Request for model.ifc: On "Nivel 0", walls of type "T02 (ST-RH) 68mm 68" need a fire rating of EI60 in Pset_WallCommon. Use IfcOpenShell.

First a look at what the model holds.

```python
import ifcopenshell
import ifcopenshell.util.element

model = ifcopenshell.open("model.ifc")
print(model.schema)
storey = next(s for s in model.by_type("IfcBuildingStorey") if s.Name == "Nivel 0")
walls = [e for e in ifcopenshell.util.element.get_decomposition(storey) if e.is_a("IfcWall")]
seen = {}
for e in walls:
    element_type = ifcopenshell.util.element.get_type(e)
    key = (element_type.Name if element_type != e and element_type else None, ifcopenshell.util.element.get_pset(e, "Pset_WallCommon", "FireRating"))
    seen[key] = seen.get(key, 0) + 1
for (name, value), count in sorted(seen.items(), key=str):
    print(count, "x", name, "|", value)
```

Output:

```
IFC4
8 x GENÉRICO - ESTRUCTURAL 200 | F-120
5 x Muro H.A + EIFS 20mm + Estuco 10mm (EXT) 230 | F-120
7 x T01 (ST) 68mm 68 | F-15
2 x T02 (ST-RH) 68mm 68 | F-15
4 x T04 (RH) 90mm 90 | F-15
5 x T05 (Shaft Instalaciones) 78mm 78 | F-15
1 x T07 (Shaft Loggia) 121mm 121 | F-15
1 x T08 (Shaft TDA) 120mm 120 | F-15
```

```python
import ifcopenshell
import ifcopenshell.api.pset
import ifcopenshell.util.element

model = ifcopenshell.open("model.ifc")

storey = next(s for s in model.by_type("IfcBuildingStorey") if s.Name == "Nivel 0")
walls = [e for e in ifcopenshell.util.element.get_decomposition(storey) if e.is_a("IfcWall")]

count = 0
for e in walls:
    element_type = ifcopenshell.util.element.get_type(e)
    if element_type in (None, e) or element_type.Name != "T02 (ST-RH) 68mm 68":
        continue
    # add_pset returns the element's existing set when there is one.
    pset = ifcopenshell.api.pset.add_pset(model, product=e, name="Pset_WallCommon")
    ifcopenshell.api.pset.edit_pset(model, pset=pset, properties={"FireRating": "EI60"})
    count += 1

print(count, "walls updated")

model.write("model_v2.ifc")
```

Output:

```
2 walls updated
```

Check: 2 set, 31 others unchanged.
